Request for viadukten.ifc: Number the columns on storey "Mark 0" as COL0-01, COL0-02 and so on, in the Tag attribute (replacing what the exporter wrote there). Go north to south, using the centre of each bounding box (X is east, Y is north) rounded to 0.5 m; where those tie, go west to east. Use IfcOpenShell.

First a look at what the model holds.

```python
import ifcopenshell
import ifcopenshell.util.element
import ifcopenshell.util.placement

model = ifcopenshell.open("viadukten.ifc")
print(model.schema)
storey = next(s for s in model.by_type("IfcBuildingStorey") if s.Name == "Mark 0")
columns = [e for e in ifcopenshell.util.element.get_decomposition(storey) if e.is_a("IfcColumn")]
for e in sorted(columns, key=lambda e: e.id()):
    origin = ifcopenshell.util.placement.get_local_placement(e.ObjectPlacement)[:3, 3]
    print(e.id(), e.Tag, e.Name, origin.round(2) + 0.0, sep=" | ")
```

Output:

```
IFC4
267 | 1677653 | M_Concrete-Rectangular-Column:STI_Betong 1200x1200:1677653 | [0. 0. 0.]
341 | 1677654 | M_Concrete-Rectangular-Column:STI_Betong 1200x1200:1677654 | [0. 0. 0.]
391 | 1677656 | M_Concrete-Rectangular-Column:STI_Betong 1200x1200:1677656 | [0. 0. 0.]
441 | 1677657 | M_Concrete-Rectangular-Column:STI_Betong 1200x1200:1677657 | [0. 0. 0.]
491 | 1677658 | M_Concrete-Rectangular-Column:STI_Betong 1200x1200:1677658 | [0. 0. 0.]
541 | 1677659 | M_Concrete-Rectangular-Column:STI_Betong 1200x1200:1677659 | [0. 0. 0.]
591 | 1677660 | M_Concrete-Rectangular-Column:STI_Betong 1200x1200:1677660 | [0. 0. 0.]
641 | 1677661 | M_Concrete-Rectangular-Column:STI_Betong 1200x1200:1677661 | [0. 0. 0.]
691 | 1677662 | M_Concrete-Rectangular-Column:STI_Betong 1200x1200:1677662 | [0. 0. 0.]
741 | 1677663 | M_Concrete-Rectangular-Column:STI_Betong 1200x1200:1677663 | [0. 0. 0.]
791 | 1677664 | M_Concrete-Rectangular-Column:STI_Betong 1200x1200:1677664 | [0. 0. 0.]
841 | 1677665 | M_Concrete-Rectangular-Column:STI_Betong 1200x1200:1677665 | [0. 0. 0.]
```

```python
import ifcopenshell
import ifcopenshell.geom
import ifcopenshell.util.element
import ifcopenshell.util.shape

model = ifcopenshell.open("viadukten.ifc")
settings = ifcopenshell.geom.settings()
settings.set("use-world-coords", True)


def centre(element):
    shape = ifcopenshell.geom.create_shape(settings, element)
    return ifcopenshell.util.shape.get_bbox_centroid(shape.geometry)


storey = next(s for s in model.by_type("IfcBuildingStorey") if s.Name == "Mark 0")
columns = [e for e in ifcopenshell.util.element.get_decomposition(storey) if e.is_a("IfcColumn")]

# Insertion points can sit at a corner or the storey origin, so sort by the geometry (in metres).
centres = {e: centre(e) for e in columns}
columns.sort(key=lambda e: (-round(centres[e][1] / 0.5), centres[e][0]))

for i, e in enumerate(columns, start=1):
    number = f"COL0-{i:02d}"
    e.Tag = number
    print(e.id(), number)

model.write("viadukten_updated.ifc")
```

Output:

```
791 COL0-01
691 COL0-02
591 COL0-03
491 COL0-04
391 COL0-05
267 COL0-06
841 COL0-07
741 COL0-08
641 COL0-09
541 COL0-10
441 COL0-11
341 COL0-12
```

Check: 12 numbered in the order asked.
